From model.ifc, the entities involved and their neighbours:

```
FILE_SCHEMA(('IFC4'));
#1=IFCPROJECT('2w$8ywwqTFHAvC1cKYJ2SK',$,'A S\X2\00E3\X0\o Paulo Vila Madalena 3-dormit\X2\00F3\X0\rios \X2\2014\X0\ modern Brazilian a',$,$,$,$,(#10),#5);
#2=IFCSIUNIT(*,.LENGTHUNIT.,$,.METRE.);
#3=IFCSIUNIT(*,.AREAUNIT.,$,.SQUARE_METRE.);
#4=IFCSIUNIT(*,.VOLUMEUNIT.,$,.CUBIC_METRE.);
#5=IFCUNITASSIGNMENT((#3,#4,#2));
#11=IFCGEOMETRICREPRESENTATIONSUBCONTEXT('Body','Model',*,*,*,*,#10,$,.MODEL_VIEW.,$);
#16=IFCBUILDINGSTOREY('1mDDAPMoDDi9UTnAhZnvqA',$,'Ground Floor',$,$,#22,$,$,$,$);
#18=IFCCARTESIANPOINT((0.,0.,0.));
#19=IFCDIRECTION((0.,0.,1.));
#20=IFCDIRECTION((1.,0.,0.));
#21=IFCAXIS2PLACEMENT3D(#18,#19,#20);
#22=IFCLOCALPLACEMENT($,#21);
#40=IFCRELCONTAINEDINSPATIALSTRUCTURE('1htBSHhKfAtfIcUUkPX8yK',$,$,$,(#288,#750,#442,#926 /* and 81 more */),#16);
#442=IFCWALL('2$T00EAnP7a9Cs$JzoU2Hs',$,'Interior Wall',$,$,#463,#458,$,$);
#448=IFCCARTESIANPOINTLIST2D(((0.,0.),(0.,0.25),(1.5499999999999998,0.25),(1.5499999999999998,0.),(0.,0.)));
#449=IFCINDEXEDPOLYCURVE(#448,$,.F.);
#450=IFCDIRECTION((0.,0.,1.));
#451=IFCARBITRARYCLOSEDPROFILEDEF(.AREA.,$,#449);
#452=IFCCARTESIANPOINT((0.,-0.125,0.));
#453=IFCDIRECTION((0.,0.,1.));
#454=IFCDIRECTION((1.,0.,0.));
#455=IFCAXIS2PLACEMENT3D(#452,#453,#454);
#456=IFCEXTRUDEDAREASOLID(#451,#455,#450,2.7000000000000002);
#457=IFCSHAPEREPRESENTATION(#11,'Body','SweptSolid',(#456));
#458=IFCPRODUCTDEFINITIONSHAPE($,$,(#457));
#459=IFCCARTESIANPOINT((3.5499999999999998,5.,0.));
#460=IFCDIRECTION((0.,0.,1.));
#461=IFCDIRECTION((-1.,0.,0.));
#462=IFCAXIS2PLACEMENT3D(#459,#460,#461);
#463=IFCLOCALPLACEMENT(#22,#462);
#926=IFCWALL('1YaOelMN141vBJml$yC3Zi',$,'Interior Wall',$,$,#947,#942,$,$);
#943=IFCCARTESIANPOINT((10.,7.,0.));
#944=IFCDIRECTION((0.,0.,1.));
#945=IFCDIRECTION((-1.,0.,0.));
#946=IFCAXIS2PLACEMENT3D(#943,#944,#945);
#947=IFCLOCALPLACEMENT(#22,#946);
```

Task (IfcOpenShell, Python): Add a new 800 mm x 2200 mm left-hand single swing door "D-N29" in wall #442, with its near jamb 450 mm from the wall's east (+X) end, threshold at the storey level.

```python
import numpy as np
import ifcopenshell
import ifcopenshell.api.feature
import ifcopenshell.api.geometry
import ifcopenshell.api.root
import ifcopenshell.api.spatial
import ifcopenshell.geom
import ifcopenshell.util.element
import ifcopenshell.util.placement
import ifcopenshell.util.representation
import ifcopenshell.util.shape
import ifcopenshell.util.unit

model = ifcopenshell.open("model.ifc")
unit_scale = ifcopenshell.util.unit.calculate_unit_scale(model)
settings = ifcopenshell.geom.settings()


def volume(element):
    """Net volume in cubic metres, openings subtracted."""
    shape = ifcopenshell.geom.create_shape(settings, element)
    return ifcopenshell.util.shape.get_volume(shape.geometry)


wall = model.by_guid("2$T00EAnP7a9Cs$JzoU2Hs")
storey = ifcopenshell.util.element.get_container(wall, ifc_class="IfcBuildingStorey")
context = ifcopenshell.util.representation.get_context(model, "Model", "Body", "MODEL_VIEW")
before = volume(wall)

width, height, from_end, sill = 0.8, 2.2, 0.45, 0.0  # metres

# The wall runs along its own X axis, and the end named is its -X end.
wall_shape = ifcopenshell.geom.create_shape(settings, wall)
x, y, z = ifcopenshell.util.shape.get_vertices(wall_shape.geometry).T
start = x.min() + from_end
face, thickness = float(y.min()), float(y.max() - y.min())
wall_matrix = ifcopenshell.util.placement.get_local_placement(wall.ObjectPlacement)
level = ifcopenshell.util.placement.get_local_placement(storey.ObjectPlacement)[2, 3]


def in_wall(x, y):
    """Placement at x, y metres in the wall's axes, at sill height."""
    matrix = wall_matrix.copy()
    matrix[:, 3] = wall_matrix @ np.array([x / unit_scale, y / unit_scale, 0.0, 1.0])
    matrix[2, 3] = level + sill / unit_scale
    return matrix


# Opening: a box that overshoots both wall faces by 50 mm.
opening = ifcopenshell.api.root.create_entity(model, ifc_class="IfcOpeningElement", predefined_type="OPENING")
box = ifcopenshell.api.geometry.add_wall_representation(
    model, context=context, length=width, height=height, thickness=thickness + 0.1
)
ifcopenshell.api.geometry.assign_representation(model, product=opening, representation=box)
ifcopenshell.api.geometry.edit_object_placement(model, product=opening, matrix=in_wall(start, face - 0.05), is_si=False)
ifcopenshell.api.feature.add_feature(model, feature=opening, element=wall)

door = ifcopenshell.api.root.create_entity(model, ifc_class="IfcDoor", name="D-N29", predefined_type="DOOR")
door.OverallWidth, door.OverallHeight = width / unit_scale, height / unit_scale
door.OperationType = "SINGLE_SWING_LEFT"
body = ifcopenshell.api.geometry.add_door_representation(
    model,
    context=context,
    overall_width=door.OverallWidth,
    overall_height=door.OverallHeight,
    operation_type="SINGLE_SWING_LEFT",
    lining_properties={"LiningDepth": thickness / unit_scale, "ThresholdDepth": thickness / unit_scale},
)
ifcopenshell.api.geometry.assign_representation(model, product=door, representation=body)
ifcopenshell.api.spatial.assign_container(model, products=[door], relating_structure=storey)
ifcopenshell.api.feature.add_filling(model, opening=opening, element=door)

# The lining spans the wall, so the door starts at the wall face.
ifcopenshell.api.geometry.edit_object_placement(model, product=door, matrix=in_wall(start, face), is_si=False)

after = volume(wall)

print(f"wall volume {before:.3f} -> {after:.3f} m3")

model.write("model_rev.ifc")
```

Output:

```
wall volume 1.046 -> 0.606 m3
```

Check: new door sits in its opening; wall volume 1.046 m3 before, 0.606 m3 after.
